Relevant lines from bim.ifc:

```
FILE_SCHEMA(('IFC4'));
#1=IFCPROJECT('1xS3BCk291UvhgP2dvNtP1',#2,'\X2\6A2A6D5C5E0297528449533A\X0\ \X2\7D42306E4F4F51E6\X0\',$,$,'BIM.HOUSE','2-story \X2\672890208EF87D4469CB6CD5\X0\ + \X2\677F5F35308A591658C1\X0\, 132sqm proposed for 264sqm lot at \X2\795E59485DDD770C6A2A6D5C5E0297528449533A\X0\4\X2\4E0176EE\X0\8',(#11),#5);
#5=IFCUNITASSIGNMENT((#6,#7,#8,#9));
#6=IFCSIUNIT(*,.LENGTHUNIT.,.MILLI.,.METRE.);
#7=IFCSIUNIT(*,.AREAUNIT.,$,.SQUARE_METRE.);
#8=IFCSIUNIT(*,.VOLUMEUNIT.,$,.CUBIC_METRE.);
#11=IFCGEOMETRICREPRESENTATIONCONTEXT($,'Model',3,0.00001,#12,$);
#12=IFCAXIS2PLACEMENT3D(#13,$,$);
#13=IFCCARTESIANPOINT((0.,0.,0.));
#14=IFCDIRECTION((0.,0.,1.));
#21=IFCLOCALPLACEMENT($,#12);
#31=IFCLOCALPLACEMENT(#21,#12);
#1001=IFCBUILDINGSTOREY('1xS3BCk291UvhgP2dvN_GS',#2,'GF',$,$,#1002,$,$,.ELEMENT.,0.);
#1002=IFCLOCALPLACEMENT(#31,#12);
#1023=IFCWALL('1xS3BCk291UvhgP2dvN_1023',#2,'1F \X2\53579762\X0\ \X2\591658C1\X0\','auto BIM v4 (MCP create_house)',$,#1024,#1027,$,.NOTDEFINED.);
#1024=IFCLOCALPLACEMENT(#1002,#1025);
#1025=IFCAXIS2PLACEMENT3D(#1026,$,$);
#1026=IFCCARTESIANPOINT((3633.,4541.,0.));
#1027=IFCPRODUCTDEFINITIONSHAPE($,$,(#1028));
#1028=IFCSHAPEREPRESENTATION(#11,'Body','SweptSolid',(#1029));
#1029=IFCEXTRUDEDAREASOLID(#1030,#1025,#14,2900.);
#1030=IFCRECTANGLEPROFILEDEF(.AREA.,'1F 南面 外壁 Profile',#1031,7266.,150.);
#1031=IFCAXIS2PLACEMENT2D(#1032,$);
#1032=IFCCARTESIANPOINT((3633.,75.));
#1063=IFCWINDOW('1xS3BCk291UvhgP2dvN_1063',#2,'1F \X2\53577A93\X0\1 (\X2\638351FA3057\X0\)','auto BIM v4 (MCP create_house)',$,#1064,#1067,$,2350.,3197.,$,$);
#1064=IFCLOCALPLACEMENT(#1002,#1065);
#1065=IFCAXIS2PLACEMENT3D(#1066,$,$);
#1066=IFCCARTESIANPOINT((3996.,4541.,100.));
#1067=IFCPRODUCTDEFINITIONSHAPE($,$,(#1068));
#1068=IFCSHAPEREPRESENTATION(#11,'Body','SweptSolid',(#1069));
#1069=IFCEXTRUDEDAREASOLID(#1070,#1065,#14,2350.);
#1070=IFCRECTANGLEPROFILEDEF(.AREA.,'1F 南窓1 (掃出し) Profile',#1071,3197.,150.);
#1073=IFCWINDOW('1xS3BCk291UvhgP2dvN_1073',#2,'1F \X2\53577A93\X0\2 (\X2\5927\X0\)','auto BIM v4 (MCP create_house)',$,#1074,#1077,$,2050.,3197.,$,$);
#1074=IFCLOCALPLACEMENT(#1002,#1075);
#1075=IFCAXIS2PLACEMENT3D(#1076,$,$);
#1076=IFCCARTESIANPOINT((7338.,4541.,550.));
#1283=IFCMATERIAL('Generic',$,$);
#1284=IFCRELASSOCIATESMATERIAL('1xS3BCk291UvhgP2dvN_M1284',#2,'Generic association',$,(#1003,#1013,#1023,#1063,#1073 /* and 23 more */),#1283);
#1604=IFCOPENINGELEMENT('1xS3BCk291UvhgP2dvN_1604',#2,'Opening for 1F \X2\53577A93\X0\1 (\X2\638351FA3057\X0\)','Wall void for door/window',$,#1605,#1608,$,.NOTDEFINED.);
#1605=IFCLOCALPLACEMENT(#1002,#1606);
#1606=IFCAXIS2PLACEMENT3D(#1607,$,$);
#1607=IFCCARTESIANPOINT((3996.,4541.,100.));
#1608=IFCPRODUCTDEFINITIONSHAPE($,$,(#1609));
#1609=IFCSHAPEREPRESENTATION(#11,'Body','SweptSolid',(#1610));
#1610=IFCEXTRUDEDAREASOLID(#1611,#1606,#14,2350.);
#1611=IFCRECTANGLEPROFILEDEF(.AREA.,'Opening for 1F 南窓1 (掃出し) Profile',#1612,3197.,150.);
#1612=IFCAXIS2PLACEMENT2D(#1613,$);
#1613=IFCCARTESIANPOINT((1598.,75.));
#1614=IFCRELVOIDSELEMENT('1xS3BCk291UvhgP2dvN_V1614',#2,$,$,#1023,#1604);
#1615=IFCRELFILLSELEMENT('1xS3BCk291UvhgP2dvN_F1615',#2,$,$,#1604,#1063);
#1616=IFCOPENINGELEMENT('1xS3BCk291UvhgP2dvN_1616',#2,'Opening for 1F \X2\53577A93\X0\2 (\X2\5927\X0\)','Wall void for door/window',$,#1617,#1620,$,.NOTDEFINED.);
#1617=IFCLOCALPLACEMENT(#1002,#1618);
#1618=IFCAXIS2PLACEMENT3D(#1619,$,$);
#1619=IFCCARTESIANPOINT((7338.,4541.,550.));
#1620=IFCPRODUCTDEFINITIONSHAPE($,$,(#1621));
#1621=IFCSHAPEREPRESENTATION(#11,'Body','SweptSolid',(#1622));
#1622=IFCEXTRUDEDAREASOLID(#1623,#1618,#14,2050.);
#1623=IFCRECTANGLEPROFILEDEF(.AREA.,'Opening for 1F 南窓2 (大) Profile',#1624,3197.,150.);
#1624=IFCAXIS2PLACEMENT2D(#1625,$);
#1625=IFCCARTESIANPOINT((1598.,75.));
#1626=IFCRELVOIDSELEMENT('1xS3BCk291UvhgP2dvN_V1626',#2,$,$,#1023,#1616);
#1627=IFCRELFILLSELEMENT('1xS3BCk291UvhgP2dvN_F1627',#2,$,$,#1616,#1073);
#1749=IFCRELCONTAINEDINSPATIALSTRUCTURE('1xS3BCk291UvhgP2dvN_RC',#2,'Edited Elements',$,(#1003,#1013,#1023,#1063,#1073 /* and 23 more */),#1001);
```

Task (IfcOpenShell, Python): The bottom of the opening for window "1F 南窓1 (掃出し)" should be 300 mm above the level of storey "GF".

```python
import numpy as np
import ifcopenshell
import ifcopenshell.api.geometry
import ifcopenshell.geom
import ifcopenshell.util.element
import ifcopenshell.util.placement
import ifcopenshell.util.shape
import ifcopenshell.util.unit

model = ifcopenshell.open("bim.ifc")
unit_scale = ifcopenshell.util.unit.calculate_unit_scale(model)

window = model.by_guid("1xS3BCk291UvhgP2dvN_1063")
opening = window.FillsVoids[0].RelatingOpeningElement
storey = ifcopenshell.util.element.get_container(window, ifc_class="IfcBuildingStorey")
level = ifcopenshell.util.placement.get_local_placement(storey.ObjectPlacement)[2, 3]

# The opening's origin need not be at the sill, so measure its lowest point.
shape = ifcopenshell.geom.create_shape(ifcopenshell.geom.settings(), opening)
bottom = ifcopenshell.util.shape.get_shape_bottom_elevation(shape, shape.geometry) / unit_scale
dz = level + 0.3 / unit_scale - bottom

shift = np.array([0.0, 0.0, dz])
# The window is not placed relative to its opening, so move both.
for product in (opening, window):
    matrix = ifcopenshell.util.placement.get_local_placement(product.ObjectPlacement)
    matrix[:3, 3] += shift
    ifcopenshell.api.geometry.edit_object_placement(model, product=product, matrix=matrix, is_si=False)

print(f"moved by {dz * unit_scale:+.3f} m")

model.write("bim_rev.ifc")
```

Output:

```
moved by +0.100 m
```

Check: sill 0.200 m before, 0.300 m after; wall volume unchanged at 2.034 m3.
